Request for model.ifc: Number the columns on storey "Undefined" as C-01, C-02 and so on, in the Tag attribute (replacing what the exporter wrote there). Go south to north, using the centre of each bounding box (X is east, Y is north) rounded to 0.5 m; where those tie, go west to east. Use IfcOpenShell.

First a look at what the model holds.

```python
import ifcopenshell
import ifcopenshell.util.element
import ifcopenshell.util.placement

model = ifcopenshell.open("model.ifc")
print(model.schema)
storey = next(s for s in model.by_type("IfcBuildingStorey") if s.Name == "Undefined")
columns = [e for e in ifcopenshell.util.element.get_decomposition(storey) if e.is_a("IfcColumn")]
for e in sorted(columns, key=lambda e: e.id()):
    origin = ifcopenshell.util.placement.get_local_placement(e.ObjectPlacement)[:3, 3]
    print(e.id(), e.Tag, e.Name, origin.round(2) + 0.0, sep=" | ")
```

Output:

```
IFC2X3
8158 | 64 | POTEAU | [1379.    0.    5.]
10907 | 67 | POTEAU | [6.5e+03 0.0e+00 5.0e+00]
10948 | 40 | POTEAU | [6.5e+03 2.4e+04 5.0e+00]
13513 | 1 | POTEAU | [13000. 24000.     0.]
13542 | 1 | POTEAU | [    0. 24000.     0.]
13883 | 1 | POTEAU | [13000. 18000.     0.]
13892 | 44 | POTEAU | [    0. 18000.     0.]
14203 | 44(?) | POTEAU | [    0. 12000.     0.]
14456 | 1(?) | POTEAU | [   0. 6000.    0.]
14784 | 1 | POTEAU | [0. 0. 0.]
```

```python
import ifcopenshell
import ifcopenshell.geom
import ifcopenshell.util.element
import ifcopenshell.util.shape

model = ifcopenshell.open("model.ifc")
settings = ifcopenshell.geom.settings()
settings.set("use-world-coords", True)


def centre(element):
    shape = ifcopenshell.geom.create_shape(settings, element)
    return ifcopenshell.util.shape.get_bbox_centroid(shape.geometry)


storey = next(s for s in model.by_type("IfcBuildingStorey") if s.Name == "Undefined")
columns = [e for e in ifcopenshell.util.element.get_decomposition(storey) if e.is_a("IfcColumn")]

# Insertion points can sit at a corner or the storey origin, so sort by the geometry (in metres).
centres = {e: centre(e) for e in columns}
columns.sort(key=lambda e: (round(centres[e][1] / 0.5), centres[e][0]))

for i, e in enumerate(columns, start=1):
    number = f"C-{i:02d}"
    e.Tag = number
    print(e.id(), number)

model.write("model_updated.ifc")
```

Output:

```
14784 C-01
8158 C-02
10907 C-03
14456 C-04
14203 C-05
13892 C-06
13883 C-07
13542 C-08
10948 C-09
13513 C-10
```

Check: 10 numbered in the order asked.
